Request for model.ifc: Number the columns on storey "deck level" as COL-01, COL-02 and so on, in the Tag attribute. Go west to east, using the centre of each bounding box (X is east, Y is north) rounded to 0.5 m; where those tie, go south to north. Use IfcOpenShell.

First a look at what the model holds.

```python
import ifcopenshell
import ifcopenshell.util.element
import ifcopenshell.util.placement

model = ifcopenshell.open("model.ifc")
print(model.schema)
storey = next(s for s in model.by_type("IfcBuildingStorey") if s.Name == "deck level")
columns = [e for e in ifcopenshell.util.element.get_decomposition(storey) if e.is_a("IfcColumn")]
for e in sorted(columns, key=lambda e: e.id()):
    origin = ifcopenshell.util.placement.get_local_placement(e.ObjectPlacement)[:3, 3]
    print(e.id(), e.Tag, e.Name, origin.round(2) + 0.0, sep=" | ")
```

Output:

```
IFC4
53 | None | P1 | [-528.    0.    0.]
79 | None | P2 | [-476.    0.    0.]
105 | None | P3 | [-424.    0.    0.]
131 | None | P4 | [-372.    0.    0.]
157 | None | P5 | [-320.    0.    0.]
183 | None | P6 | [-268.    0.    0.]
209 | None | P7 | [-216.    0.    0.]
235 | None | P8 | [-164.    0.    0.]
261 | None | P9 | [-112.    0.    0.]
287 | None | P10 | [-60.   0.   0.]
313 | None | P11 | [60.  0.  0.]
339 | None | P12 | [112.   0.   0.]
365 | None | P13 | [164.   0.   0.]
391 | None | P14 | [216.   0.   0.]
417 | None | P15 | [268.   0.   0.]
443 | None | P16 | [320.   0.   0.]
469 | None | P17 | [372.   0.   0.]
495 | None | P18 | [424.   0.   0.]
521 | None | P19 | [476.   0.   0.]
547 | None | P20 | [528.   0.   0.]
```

```python
import ifcopenshell
import ifcopenshell.geom
import ifcopenshell.util.element
import ifcopenshell.util.shape

model = ifcopenshell.open("model.ifc")
settings = ifcopenshell.geom.settings()
settings.set("use-world-coords", True)


def centre(element):
    shape = ifcopenshell.geom.create_shape(settings, element)
    return ifcopenshell.util.shape.get_bbox_centroid(shape.geometry)


storey = next(s for s in model.by_type("IfcBuildingStorey") if s.Name == "deck level")
columns = [e for e in ifcopenshell.util.element.get_decomposition(storey) if e.is_a("IfcColumn")]

# Insertion points can sit at a corner or the storey origin, so sort by the geometry (in metres).
centres = {e: centre(e) for e in columns}
columns.sort(key=lambda e: (round(centres[e][0] / 0.5), centres[e][1]))

for i, e in enumerate(columns, start=1):
    number = f"COL-{i:02d}"
    e.Tag = number
    print(e.id(), number)

model.write("model_v2.ifc")
```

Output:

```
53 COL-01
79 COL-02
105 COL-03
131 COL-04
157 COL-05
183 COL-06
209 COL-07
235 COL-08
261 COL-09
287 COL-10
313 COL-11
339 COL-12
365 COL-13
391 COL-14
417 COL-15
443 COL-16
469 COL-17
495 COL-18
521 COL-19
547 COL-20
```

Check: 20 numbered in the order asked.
